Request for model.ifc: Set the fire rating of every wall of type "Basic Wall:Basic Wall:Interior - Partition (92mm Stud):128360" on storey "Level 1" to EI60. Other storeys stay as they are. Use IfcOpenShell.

First a look at what the model holds.

```python
import ifcopenshell
import ifcopenshell.util.element

model = ifcopenshell.open("model.ifc")
print(model.schema)
storey = next(s for s in model.by_type("IfcBuildingStorey") if s.Name == "Level 1")
walls = [e for e in ifcopenshell.util.element.get_decomposition(storey) if e.is_a("IfcWall")]
seen = {}
for e in walls:
    element_type = ifcopenshell.util.element.get_type(e)
    key = (element_type.Name if element_type != e and element_type else None, ifcopenshell.util.element.get_pset(e, "Pset_WallCommon", "FireRating"))
    seen[key] = seen.get(key, 0) + 1
for (name, value), count in sorted(seen.items(), key=str):
    print(count, "x", name, "|", value)
```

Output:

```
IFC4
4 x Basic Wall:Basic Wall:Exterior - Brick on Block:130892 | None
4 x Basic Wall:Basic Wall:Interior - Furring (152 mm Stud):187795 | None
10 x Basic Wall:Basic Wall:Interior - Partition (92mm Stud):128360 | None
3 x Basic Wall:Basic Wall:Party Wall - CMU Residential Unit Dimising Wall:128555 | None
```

```python
import ifcopenshell
import ifcopenshell.api.pset
import ifcopenshell.util.element

model = ifcopenshell.open("model.ifc")

storey = next(s for s in model.by_type("IfcBuildingStorey") if s.Name == "Level 1")
walls = [e for e in ifcopenshell.util.element.get_decomposition(storey) if e.is_a("IfcWall")]

count = 0
for e in walls:
    element_type = ifcopenshell.util.element.get_type(e)
    if element_type in (None, e) or element_type.Name != "Basic Wall:Basic Wall:Interior - Partition (92mm Stud):128360":
        continue
    # add_pset returns the element's existing set when there is one.
    pset = ifcopenshell.api.pset.add_pset(model, product=e, name="Pset_WallCommon")
    ifcopenshell.api.pset.edit_pset(model, pset=pset, properties={"FireRating": "EI60"})
    count += 1

print(count, "walls updated")

model.write("model_updated.ifc")
```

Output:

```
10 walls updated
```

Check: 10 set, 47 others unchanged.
